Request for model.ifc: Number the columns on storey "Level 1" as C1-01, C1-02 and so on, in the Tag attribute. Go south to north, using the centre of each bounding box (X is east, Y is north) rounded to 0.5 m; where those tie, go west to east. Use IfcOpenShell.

First a look at what the model holds.

```python
import ifcopenshell
import ifcopenshell.util.element
import ifcopenshell.util.placement

model = ifcopenshell.open("model.ifc")
print(model.schema)
storey = next(s for s in model.by_type("IfcBuildingStorey") if s.Name == "Level 1")
columns = [e for e in ifcopenshell.util.element.get_decomposition(storey) if e.is_a("IfcColumn")]
for e in sorted(columns, key=lambda e: e.id()):
    origin = ifcopenshell.util.placement.get_local_placement(e.ObjectPlacement)[:3, 3]
    print(e.id(), e.Tag, e.Name, origin.round(2) + 0.0, sep=" | ")
```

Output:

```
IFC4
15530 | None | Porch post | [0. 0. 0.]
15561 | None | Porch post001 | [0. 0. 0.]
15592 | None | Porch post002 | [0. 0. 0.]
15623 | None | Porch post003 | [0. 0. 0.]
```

```python
import ifcopenshell
import ifcopenshell.geom
import ifcopenshell.util.element
import ifcopenshell.util.shape

model = ifcopenshell.open("model.ifc")
settings = ifcopenshell.geom.settings()
settings.set("use-world-coords", True)


def centre(element):
    shape = ifcopenshell.geom.create_shape(settings, element)
    return ifcopenshell.util.shape.get_bbox_centroid(shape.geometry)


storey = next(s for s in model.by_type("IfcBuildingStorey") if s.Name == "Level 1")
columns = [e for e in ifcopenshell.util.element.get_decomposition(storey) if e.is_a("IfcColumn")]

# Insertion points can sit at a corner or the storey origin, so sort by the geometry (in metres).
centres = {e: centre(e) for e in columns}
columns.sort(key=lambda e: (round(centres[e][1] / 0.5), centres[e][0]))

for i, e in enumerate(columns, start=1):
    number = f"C1-{i:02d}"
    e.Tag = number
    print(e.id(), number)

model.write("model_rev.ifc")
```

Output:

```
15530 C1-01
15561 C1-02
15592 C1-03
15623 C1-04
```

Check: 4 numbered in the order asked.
